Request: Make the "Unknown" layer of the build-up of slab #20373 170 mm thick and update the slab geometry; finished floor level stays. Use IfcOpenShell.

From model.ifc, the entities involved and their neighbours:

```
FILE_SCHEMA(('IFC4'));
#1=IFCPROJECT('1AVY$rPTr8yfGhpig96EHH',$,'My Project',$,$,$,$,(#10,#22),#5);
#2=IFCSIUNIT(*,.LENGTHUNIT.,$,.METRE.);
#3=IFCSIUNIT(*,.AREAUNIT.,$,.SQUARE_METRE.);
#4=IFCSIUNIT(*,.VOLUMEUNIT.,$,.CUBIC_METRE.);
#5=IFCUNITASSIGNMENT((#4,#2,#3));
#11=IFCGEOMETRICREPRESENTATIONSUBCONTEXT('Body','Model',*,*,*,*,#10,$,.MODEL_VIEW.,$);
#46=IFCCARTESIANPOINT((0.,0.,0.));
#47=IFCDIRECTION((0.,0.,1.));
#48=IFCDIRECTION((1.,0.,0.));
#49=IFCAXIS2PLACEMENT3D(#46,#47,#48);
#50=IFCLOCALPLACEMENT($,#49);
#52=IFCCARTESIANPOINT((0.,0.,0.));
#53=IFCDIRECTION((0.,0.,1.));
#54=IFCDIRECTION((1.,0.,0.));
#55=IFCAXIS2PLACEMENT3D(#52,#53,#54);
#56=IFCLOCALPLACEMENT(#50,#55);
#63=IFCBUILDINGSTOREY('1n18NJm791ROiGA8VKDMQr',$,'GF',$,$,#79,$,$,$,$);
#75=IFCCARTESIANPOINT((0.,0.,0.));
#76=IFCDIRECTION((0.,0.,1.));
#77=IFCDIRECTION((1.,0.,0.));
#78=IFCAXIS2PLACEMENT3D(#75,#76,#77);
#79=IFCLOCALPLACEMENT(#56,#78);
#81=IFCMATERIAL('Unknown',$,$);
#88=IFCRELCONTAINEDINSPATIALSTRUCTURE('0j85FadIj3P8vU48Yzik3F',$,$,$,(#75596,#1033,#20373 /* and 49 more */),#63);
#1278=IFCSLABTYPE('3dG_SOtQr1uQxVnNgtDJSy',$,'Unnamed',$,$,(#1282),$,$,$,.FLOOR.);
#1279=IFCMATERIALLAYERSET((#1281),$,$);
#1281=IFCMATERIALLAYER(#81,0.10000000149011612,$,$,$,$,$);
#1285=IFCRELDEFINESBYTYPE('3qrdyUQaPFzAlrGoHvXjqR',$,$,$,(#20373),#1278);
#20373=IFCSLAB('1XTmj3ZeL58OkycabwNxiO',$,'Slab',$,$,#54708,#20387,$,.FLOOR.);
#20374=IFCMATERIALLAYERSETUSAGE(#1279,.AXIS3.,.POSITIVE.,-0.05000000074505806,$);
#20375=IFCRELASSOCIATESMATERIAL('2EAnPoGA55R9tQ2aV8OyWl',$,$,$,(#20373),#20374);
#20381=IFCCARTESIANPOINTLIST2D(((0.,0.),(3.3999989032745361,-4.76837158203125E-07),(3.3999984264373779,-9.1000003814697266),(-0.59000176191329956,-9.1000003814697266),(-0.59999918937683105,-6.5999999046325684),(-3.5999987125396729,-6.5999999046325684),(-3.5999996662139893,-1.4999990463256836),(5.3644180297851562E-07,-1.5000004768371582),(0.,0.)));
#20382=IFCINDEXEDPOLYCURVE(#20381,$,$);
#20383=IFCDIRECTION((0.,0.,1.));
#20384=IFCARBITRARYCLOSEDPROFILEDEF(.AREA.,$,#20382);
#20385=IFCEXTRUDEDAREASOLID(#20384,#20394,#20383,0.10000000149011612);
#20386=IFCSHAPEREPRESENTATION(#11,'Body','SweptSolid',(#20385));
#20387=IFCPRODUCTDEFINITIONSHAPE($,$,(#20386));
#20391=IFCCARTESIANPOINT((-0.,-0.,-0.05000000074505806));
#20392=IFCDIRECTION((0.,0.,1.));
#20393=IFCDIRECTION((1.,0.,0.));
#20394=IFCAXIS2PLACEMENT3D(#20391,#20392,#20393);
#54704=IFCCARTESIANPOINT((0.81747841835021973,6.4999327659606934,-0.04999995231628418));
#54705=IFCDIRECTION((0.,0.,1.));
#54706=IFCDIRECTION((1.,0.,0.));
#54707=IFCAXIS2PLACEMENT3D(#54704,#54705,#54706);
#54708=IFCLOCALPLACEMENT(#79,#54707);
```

```python
import ifcopenshell
import ifcopenshell.util.element
import ifcopenshell.util.representation

model = ifcopenshell.open("model.ifc")

layer_set = model.by_id(1279)
layer = next(l for l in layer_set.MaterialLayers if l.Material and l.Material.Name == "Unknown")
change = 0.17 - layer.LayerThickness
layer.LayerThickness += change

# Geometry does not follow the layer set by itself.
slabs = [e for e in ifcopenshell.util.element.get_elements_by_material(model, layer_set) if e.is_a("IfcSlab")]
for slab in sorted(slabs, key=lambda e: e.id()):
    body = ifcopenshell.util.representation.get_representation(slab, "Model", "Body")
    solid = body.Items[0]
    old_depth = solid.Depth
    solid.Depth += change
    # Extruded upwards: lower the start of the extrusion so the top stays.
    x, y, z = solid.Position.Location.Coordinates
    solid.Position.Location = model.createIfcCartesianPoint((x, y, z - change))
    print(slab.id(), f"{old_depth:g} -> {solid.Depth:g}")

# The layers are counted up from the underside, which has moved.
for usage in {ifcopenshell.util.element.get_material(slab) for slab in slabs}:
    usage.OffsetFromReferenceLine -= change

model.write("model_rev.ifc")
```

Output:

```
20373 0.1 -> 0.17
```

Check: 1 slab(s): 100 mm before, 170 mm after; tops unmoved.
